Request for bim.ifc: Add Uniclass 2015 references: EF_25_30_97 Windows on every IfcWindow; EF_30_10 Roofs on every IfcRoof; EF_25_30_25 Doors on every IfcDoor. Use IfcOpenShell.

First a look at what the model holds.

```python
import ifcopenshell

model = ifcopenshell.open("bim.ifc")
print(model.schema)
print("classifications:", [c.Name for c in model.by_type("IfcClassification")])
for ifc_class in ("IfcDoor", "IfcRoof", "IfcStair", "IfcWall", "IfcWindow"):
    print(ifc_class, len(model.by_type(ifc_class)))
```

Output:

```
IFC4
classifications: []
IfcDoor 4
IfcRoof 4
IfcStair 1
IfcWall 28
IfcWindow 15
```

```python
import ifcopenshell
import ifcopenshell.api.classification

model = ifcopenshell.open("bim.ifc")

system = ifcopenshell.api.classification.add_classification(model, classification="Uniclass 2015")

codes = {
    "IfcWindow": ("EF_25_30_97", "Windows"),
    "IfcRoof": ("EF_30_10", "Roofs"),
    "IfcDoor": ("EF_25_30_25", "Doors"),
}
for ifc_class, (code, name) in codes.items():
    products = model.by_type(ifc_class)
    ifcopenshell.api.classification.add_reference(
        model, products=products, classification=system, identification=code, name=name
    )
    print(code, len(products))

model.write("bim_rev.ifc")
```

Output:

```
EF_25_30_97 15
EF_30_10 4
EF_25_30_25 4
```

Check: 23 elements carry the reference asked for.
